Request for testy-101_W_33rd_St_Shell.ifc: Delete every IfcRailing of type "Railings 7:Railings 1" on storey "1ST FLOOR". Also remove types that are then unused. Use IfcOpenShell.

First a look at what the model holds.

```python
import ifcopenshell
import ifcopenshell.util.element

model = ifcopenshell.open("testy-101_W_33rd_St_Shell.ifc")
print(model.schema)
storey = next(s for s in model.by_type("IfcBuildingStorey") if s.Name == "1ST FLOOR")
railings = [e for e in ifcopenshell.util.element.get_decomposition(storey) if e.is_a("IfcRailing")]
seen = {}
for e in railings:
    element_type = ifcopenshell.util.element.get_type(e)
    name = element_type.Name if element_type not in (None, e) else None
    seen[name] = seen.get(name, 0) + 1
for name, count in sorted(seen.items(), key=str):
    print(count, "x", name)
```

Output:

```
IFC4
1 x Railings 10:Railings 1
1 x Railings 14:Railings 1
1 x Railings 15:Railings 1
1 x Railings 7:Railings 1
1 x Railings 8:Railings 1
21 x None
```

```python
import ifcopenshell
import ifcopenshell.api.root
import ifcopenshell.util.element

model = ifcopenshell.open("testy-101_W_33rd_St_Shell.ifc")

storey = next(s for s in model.by_type("IfcBuildingStorey") if s.Name == "1ST FLOOR")
railings = [e for e in ifcopenshell.util.element.get_decomposition(storey) if e.is_a("IfcRailing")]
targets = [e for e in railings if (t := ifcopenshell.util.element.get_type(e)) not in (None, e) and t.Name == "Railings 7:Railings 1"]
types = {ifcopenshell.util.element.get_type(e) for e in targets} - {None, *targets}

for e in targets:
    ifcopenshell.api.root.remove_product(model, product=e)
print(len(targets), "removed")

unused = [t for t in types if not ifcopenshell.util.element.get_types(t)]
for t in unused:
    ifcopenshell.api.root.remove_product(model, product=t)
print(len(unused), "unused types removed")

model.write("testy-101_W_33rd_St_Shell_updated.ifc")
```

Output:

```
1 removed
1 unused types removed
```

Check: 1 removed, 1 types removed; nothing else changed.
